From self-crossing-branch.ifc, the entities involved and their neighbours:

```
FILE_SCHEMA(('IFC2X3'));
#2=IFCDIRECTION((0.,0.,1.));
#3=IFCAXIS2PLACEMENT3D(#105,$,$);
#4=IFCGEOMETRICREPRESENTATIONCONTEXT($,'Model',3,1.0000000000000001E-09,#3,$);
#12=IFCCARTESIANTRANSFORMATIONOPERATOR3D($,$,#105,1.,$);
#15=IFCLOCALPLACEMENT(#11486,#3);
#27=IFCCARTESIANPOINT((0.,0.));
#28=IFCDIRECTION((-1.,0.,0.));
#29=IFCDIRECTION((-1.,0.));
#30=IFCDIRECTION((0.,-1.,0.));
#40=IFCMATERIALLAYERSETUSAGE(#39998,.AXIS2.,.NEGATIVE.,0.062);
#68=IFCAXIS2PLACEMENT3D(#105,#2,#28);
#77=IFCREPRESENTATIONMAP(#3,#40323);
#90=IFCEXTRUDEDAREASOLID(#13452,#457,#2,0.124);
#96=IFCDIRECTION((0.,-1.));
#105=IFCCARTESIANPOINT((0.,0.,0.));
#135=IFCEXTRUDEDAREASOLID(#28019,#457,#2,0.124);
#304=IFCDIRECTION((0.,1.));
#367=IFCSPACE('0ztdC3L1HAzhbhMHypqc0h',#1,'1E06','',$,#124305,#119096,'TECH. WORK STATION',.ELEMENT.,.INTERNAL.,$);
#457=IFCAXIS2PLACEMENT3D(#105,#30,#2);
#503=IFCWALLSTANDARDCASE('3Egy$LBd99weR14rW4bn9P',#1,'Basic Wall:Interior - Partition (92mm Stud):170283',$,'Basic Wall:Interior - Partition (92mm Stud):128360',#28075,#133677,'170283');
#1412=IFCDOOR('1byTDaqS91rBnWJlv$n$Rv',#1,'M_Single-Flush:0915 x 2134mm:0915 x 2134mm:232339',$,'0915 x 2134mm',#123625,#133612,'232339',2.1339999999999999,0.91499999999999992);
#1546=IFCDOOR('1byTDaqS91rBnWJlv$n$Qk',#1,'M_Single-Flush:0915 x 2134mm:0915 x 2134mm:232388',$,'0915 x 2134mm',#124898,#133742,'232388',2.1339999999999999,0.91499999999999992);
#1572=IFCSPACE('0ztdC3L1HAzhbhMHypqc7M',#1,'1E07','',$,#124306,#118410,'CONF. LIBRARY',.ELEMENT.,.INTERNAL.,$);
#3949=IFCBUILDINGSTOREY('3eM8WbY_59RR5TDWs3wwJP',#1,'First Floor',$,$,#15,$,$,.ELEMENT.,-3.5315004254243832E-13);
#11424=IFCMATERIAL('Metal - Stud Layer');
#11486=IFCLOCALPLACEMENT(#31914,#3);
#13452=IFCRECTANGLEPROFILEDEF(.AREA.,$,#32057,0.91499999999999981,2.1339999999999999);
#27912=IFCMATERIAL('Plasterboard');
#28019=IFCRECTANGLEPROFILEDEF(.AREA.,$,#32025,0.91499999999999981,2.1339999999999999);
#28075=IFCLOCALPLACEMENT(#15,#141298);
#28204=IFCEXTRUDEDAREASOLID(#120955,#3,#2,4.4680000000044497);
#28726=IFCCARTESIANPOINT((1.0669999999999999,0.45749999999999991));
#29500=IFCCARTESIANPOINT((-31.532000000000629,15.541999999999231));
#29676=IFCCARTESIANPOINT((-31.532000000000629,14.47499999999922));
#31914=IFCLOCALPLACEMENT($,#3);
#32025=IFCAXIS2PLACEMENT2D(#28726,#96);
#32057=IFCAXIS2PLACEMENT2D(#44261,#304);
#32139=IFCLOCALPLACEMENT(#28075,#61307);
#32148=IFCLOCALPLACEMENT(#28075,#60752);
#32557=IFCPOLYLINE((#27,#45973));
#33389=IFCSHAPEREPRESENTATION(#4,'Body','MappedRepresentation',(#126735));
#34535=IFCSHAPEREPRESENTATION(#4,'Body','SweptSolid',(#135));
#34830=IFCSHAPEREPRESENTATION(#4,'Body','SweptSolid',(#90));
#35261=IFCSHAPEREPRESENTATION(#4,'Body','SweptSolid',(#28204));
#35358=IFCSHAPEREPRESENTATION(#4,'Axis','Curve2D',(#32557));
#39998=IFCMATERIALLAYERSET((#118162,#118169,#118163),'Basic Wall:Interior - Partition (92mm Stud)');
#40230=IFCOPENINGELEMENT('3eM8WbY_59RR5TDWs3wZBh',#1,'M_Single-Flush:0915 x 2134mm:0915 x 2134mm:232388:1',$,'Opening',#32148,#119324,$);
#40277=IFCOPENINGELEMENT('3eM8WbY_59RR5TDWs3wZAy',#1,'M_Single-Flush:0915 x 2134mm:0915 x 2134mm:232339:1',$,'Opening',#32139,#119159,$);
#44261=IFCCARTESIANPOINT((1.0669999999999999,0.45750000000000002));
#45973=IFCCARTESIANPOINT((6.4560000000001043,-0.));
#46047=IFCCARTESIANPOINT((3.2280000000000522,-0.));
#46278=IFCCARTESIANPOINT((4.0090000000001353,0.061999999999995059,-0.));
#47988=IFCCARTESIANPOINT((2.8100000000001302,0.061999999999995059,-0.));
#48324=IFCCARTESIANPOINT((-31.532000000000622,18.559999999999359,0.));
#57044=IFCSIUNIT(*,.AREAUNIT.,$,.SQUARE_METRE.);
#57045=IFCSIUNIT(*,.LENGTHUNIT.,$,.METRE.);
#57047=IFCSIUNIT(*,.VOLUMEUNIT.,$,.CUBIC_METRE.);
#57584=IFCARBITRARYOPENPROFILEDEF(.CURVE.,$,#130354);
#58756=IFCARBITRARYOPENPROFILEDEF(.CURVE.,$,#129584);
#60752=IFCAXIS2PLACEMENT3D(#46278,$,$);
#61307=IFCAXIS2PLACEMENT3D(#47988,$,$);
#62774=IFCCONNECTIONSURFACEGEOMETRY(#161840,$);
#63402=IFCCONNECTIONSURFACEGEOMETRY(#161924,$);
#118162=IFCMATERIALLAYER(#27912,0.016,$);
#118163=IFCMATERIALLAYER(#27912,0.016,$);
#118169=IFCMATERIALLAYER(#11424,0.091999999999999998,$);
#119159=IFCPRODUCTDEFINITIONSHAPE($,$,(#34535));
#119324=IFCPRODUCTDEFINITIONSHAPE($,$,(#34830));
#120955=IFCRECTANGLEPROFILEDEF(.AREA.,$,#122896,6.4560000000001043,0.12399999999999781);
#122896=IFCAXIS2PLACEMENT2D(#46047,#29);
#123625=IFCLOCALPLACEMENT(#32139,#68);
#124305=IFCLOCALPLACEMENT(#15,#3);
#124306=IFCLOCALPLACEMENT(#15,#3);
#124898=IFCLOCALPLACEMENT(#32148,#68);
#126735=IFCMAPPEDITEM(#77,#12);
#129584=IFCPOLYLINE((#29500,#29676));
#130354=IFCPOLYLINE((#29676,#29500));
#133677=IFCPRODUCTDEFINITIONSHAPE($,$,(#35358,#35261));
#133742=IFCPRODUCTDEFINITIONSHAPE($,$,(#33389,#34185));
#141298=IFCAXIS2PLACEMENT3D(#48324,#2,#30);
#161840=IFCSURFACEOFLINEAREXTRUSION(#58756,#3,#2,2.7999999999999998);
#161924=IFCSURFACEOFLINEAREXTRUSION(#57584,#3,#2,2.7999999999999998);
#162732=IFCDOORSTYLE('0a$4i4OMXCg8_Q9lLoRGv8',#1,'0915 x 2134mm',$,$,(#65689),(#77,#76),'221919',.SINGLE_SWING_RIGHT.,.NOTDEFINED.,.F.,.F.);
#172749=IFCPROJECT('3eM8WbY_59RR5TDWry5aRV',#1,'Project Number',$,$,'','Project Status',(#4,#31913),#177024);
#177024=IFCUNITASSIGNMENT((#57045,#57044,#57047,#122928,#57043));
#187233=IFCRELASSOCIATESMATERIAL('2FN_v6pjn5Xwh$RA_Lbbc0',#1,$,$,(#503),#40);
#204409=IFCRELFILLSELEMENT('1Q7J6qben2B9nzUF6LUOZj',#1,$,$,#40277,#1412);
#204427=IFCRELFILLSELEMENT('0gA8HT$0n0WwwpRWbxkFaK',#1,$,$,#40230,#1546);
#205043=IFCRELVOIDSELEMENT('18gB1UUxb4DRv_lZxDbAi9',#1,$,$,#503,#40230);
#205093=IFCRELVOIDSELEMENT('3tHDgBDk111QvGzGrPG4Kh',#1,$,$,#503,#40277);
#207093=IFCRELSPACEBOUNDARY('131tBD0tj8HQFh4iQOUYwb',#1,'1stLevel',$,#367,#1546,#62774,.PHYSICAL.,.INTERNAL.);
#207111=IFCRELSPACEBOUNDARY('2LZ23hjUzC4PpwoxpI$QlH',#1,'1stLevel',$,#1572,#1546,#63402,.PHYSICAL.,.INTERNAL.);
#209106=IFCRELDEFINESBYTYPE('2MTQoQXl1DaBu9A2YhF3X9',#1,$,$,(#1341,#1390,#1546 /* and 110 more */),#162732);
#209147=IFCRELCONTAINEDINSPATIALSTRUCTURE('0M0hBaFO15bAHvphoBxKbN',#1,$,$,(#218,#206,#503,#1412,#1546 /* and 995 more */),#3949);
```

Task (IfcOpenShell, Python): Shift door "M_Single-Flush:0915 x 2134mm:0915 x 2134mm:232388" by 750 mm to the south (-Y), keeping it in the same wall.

```python
import numpy as np
import ifcopenshell
import ifcopenshell.api.geometry
import ifcopenshell.util.placement

model = ifcopenshell.open("self-crossing-branch.ifc")

door = model.by_guid("1byTDaqS91rBnWJlv$n$Qk")
opening = door.FillsVoids[0].RelatingOpeningElement
wall = opening.VoidsElements[0].RelatingBuildingElement

wall_matrix = ifcopenshell.util.placement.get_local_placement(wall.ObjectPlacement)
shift = wall_matrix[:3, 0] * 0.75
before = ifcopenshell.util.placement.get_local_placement(door.ObjectPlacement)[:3, 3].copy()

# The door is placed relative to its opening, so it follows when the opening moves.
matrix = ifcopenshell.util.placement.get_local_placement(opening.ObjectPlacement)
matrix[:3, 3] += shift
ifcopenshell.api.geometry.edit_object_placement(
    model, product=opening, matrix=matrix, is_si=False, should_transform_children=True
)

# Space boundary surfaces are stored in each space's coordinates; move them too.
for rel in door.ProvidesBoundaries:
    if not rel.ConnectionGeometry:
        continue
    surface = rel.ConnectionGeometry.SurfaceOnRelatingElement
    space_matrix = ifcopenshell.util.placement.get_local_placement(rel.RelatingSpace.ObjectPlacement)
    point = np.array(surface.Position.Location.Coordinates) + space_matrix[:3, :3].T @ shift
    surface.Position = model.createIfcAxis2Placement3D(
        model.createIfcCartesianPoint(point.tolist()), surface.Position.Axis, surface.Position.RefDirection
    )

after = ifcopenshell.util.placement.get_local_placement(door.ObjectPlacement)[:3, 3]
print("door moved by", (after - before).round(3) + 0.0)

model.write("self-crossing-branch_updated.ifc")
```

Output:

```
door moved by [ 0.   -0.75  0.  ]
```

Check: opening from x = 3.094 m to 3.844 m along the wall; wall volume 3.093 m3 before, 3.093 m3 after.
